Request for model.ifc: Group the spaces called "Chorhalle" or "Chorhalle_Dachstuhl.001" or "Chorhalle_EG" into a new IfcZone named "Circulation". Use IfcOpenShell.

First a look at what the model holds.

```python
import ifcopenshell

model = ifcopenshell.open("model.ifc")
print(model.schema)
seen = {}
for space in model.by_type("IfcSpace"):
    seen[space.Name] = seen.get(space.Name, 0) + 1
for name, count in sorted(seen.items(), key=str):
    print(count, "x", name)
print("zones:", [z.Name for z in model.by_type("IfcZone")][:20])
```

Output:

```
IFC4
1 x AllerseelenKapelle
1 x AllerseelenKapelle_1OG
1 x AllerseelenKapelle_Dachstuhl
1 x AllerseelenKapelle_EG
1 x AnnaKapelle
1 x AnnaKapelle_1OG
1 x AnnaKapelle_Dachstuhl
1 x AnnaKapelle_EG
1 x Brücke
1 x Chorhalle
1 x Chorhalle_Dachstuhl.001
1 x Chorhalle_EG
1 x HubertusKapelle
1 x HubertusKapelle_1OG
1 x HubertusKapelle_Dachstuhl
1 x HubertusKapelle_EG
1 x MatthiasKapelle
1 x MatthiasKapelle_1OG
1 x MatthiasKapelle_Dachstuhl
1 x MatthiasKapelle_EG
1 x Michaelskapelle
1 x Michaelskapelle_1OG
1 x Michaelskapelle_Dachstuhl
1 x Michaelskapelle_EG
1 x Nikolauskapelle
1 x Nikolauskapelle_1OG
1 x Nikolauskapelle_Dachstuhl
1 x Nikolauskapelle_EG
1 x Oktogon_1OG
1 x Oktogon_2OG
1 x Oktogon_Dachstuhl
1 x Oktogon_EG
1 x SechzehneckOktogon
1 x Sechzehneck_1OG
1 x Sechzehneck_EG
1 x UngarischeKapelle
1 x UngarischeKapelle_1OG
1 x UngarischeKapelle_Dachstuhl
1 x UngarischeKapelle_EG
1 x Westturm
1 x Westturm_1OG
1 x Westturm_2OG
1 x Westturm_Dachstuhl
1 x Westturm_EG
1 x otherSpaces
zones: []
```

```python
import ifcopenshell
import ifcopenshell.api.group
import ifcopenshell.api.root

model = ifcopenshell.open("model.ifc")

names = {"Chorhalle", "Chorhalle_Dachstuhl.001", "Chorhalle_EG"}
spaces = [s for s in model.by_type("IfcSpace") if s.Name in names]

zone = ifcopenshell.api.root.create_entity(model, ifc_class="IfcZone", name="Circulation")
ifcopenshell.api.group.assign_group(model, products=spaces, group=zone)
print(len(spaces), "spaces in", zone.Name)

model.write("model_edited.ifc")
```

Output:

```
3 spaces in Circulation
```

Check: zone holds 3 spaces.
